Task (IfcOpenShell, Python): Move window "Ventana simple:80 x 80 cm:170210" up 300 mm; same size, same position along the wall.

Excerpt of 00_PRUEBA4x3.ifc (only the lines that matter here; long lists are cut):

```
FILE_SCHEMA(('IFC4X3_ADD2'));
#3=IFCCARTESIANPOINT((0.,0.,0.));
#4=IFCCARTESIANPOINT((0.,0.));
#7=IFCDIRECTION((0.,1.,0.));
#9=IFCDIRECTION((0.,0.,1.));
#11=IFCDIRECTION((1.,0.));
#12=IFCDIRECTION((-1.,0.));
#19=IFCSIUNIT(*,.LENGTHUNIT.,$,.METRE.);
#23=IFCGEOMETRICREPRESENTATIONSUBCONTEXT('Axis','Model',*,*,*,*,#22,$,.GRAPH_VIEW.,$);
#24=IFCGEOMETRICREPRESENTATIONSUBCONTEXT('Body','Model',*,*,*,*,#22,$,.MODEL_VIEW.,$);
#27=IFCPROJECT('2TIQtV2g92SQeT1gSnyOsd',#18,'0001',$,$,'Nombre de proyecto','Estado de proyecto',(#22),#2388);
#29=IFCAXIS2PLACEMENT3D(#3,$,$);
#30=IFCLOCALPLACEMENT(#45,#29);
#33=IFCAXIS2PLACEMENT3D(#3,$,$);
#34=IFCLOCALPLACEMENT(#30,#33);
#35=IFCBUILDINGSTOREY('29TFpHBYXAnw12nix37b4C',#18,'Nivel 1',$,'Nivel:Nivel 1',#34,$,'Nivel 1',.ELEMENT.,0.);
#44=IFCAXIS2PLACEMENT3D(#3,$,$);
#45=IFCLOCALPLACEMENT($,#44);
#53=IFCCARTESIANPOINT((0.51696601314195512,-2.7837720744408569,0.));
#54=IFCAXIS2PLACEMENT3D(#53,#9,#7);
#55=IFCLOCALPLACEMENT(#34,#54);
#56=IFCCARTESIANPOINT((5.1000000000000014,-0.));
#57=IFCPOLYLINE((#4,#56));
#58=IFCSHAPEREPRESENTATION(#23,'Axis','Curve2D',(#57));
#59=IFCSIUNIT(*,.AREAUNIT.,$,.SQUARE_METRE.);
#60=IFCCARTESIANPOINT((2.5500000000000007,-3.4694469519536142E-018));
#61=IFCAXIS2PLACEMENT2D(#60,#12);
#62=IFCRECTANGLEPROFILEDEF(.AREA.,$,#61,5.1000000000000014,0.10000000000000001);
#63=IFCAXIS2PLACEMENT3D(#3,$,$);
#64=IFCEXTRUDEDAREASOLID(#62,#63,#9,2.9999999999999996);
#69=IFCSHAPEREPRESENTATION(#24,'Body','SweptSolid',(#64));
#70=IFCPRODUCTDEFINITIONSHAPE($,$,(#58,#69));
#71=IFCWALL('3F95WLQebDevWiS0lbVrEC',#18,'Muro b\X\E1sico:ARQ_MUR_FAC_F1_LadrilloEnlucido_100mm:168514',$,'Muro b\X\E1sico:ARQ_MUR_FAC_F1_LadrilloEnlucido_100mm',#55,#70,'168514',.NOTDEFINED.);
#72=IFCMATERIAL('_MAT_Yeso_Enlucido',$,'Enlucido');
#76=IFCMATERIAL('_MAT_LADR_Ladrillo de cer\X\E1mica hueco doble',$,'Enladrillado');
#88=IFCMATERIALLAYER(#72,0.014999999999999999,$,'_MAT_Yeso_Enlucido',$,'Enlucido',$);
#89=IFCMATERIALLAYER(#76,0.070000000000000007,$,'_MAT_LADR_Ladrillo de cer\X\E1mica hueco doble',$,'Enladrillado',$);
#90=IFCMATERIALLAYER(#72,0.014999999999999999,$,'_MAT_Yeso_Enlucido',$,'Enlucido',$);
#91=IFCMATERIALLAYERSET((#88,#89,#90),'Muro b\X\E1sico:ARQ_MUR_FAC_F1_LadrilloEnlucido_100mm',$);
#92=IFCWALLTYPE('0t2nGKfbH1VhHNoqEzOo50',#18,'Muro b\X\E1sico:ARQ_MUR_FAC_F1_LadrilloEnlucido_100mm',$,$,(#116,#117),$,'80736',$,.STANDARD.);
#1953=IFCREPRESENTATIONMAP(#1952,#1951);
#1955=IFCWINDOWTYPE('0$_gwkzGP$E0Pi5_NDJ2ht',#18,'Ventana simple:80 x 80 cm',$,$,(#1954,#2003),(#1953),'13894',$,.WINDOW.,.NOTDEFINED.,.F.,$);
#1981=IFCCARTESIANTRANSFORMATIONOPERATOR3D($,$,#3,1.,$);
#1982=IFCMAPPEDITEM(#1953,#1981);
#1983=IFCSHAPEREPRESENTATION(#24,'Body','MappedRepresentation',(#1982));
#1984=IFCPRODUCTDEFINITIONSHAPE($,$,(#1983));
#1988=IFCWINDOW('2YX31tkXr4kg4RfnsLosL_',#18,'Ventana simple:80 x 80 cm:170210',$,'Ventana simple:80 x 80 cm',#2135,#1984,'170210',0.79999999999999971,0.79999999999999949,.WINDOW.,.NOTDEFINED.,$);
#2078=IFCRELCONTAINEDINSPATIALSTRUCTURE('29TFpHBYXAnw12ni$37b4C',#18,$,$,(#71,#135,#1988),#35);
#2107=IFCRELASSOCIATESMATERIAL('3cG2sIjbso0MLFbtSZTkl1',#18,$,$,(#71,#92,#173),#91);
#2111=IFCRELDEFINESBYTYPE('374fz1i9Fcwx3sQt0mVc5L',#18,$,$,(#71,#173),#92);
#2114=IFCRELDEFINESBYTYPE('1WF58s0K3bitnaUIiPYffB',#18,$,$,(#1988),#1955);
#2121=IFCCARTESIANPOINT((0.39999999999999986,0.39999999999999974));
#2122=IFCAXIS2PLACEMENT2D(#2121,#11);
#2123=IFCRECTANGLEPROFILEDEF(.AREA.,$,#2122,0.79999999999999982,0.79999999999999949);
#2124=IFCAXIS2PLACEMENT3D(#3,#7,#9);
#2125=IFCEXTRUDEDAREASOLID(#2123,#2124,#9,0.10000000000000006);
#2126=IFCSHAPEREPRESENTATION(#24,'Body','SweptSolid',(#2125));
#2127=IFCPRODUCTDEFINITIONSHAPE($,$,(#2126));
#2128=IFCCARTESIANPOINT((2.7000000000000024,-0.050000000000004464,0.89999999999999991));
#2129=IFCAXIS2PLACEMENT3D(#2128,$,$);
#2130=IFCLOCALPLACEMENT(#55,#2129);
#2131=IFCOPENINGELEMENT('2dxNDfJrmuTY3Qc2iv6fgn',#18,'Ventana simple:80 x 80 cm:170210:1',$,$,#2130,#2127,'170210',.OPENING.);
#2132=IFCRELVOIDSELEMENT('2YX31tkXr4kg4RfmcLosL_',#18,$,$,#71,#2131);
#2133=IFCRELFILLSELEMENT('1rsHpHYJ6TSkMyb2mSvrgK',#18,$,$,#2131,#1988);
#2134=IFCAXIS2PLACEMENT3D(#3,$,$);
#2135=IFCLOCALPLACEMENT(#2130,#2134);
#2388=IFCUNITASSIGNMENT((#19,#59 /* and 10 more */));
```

```python
import numpy as np
import ifcopenshell
import ifcopenshell.api.geometry
import ifcopenshell.util.placement
import ifcopenshell.util.unit

model = ifcopenshell.open("00_PRUEBA4x3.ifc")
unit_scale = ifcopenshell.util.unit.calculate_unit_scale(model)

window = model.by_id(1988)
opening = window.FillsVoids[0].RelatingOpeningElement
dz = 0.3 / unit_scale

shift = np.array([0.0, 0.0, dz])
# The window is placed relative to its opening, so it follows when the opening moves.
matrix = ifcopenshell.util.placement.get_local_placement(opening.ObjectPlacement)
matrix[:3, 3] += shift
ifcopenshell.api.geometry.edit_object_placement(
    model, product=opening, matrix=matrix, is_si=False, should_transform_children=True
)

print(f"moved by {dz * unit_scale:+.3f} m")

model.write("00_PRUEBA4x3-out.ifc")
```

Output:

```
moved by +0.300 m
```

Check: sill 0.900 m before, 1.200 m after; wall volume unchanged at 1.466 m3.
